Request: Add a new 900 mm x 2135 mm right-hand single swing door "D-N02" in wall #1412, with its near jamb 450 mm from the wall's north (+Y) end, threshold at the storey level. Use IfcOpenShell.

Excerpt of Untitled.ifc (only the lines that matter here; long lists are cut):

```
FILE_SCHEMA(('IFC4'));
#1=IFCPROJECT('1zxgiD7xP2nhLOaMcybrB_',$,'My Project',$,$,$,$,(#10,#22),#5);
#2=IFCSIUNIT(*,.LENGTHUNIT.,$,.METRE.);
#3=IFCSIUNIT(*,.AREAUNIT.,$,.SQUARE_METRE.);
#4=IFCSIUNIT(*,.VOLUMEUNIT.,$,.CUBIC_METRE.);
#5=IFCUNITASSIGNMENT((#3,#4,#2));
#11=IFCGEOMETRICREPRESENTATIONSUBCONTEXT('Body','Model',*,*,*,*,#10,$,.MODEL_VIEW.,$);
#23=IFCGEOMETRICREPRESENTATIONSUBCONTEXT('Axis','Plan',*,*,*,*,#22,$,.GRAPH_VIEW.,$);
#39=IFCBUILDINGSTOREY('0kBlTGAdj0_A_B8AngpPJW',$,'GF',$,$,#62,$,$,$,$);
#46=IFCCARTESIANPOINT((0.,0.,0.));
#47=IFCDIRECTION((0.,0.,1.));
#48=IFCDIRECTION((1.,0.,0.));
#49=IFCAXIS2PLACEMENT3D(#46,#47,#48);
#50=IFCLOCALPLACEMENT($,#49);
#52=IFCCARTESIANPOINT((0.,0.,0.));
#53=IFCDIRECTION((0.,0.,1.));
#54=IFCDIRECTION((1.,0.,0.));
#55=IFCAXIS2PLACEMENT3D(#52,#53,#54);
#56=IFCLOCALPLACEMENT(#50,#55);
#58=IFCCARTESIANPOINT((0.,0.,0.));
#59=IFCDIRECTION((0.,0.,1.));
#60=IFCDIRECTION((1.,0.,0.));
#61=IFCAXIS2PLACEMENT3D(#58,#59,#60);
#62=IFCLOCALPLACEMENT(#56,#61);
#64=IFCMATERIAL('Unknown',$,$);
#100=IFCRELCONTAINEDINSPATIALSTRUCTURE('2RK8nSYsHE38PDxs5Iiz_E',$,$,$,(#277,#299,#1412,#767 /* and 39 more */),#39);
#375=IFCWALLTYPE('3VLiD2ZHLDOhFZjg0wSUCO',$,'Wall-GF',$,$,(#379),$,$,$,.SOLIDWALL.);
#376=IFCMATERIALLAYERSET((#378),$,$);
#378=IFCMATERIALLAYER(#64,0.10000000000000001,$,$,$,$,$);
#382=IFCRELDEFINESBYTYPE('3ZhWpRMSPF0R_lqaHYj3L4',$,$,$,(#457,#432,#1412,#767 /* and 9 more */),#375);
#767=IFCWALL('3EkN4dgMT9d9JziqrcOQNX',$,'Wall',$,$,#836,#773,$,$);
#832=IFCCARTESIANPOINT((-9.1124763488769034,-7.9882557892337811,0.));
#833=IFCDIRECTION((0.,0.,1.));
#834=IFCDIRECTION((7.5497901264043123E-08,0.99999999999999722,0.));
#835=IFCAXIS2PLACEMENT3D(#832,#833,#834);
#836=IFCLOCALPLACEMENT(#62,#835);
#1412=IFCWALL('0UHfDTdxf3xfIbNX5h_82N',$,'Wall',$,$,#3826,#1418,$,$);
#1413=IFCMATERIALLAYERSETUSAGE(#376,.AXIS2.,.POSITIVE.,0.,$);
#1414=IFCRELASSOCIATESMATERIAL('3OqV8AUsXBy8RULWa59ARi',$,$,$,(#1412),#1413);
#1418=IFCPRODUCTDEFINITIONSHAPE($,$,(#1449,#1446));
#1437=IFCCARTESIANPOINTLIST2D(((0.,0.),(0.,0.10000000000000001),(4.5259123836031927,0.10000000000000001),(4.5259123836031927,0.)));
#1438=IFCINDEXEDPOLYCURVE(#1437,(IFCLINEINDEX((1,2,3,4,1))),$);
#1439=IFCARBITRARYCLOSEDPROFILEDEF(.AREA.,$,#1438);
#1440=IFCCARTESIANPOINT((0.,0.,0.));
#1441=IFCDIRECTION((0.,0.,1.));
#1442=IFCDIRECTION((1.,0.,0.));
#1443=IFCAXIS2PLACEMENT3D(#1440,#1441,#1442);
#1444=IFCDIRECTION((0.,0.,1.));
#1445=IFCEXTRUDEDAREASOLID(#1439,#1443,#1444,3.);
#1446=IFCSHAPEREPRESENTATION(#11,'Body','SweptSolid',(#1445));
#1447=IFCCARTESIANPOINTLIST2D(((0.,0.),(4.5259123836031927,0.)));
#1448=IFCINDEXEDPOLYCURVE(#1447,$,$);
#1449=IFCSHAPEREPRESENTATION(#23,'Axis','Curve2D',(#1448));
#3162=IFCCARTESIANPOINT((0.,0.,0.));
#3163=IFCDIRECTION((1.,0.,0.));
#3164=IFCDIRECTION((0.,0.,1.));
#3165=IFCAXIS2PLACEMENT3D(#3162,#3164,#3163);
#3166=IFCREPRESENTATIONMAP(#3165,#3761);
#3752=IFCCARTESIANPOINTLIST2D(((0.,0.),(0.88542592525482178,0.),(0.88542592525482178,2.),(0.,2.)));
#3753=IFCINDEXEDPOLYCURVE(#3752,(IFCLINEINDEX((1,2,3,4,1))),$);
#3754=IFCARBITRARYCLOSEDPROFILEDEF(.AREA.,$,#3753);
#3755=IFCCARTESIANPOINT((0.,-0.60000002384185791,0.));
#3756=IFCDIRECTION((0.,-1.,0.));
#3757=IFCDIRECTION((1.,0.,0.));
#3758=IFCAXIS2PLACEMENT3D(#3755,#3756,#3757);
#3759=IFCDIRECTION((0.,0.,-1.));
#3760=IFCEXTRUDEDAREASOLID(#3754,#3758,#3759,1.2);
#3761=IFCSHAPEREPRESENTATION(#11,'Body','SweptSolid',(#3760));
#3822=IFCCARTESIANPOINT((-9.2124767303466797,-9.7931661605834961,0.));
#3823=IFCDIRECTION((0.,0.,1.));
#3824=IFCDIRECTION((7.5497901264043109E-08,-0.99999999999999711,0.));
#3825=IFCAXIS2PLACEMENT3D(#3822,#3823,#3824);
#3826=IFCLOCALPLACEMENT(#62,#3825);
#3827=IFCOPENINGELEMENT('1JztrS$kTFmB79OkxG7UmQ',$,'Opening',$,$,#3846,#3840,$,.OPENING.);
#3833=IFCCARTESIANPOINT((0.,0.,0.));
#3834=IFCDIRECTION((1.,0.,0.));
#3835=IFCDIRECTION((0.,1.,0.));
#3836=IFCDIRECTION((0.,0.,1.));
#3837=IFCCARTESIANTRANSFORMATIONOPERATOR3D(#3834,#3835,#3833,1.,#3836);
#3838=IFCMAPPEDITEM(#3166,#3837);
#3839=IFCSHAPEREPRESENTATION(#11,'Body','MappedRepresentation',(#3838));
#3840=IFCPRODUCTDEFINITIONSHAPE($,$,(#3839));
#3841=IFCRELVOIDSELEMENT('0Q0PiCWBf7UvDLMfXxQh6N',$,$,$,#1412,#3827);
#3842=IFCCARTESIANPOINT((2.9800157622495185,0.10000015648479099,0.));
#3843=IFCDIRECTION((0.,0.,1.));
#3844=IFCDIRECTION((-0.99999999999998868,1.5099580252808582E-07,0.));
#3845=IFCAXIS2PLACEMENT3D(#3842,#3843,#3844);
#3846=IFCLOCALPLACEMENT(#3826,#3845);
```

```python
import numpy as np
import ifcopenshell
import ifcopenshell.api.feature
import ifcopenshell.api.geometry
import ifcopenshell.api.root
import ifcopenshell.api.spatial
import ifcopenshell.geom
import ifcopenshell.util.element
import ifcopenshell.util.placement
import ifcopenshell.util.representation
import ifcopenshell.util.shape
import ifcopenshell.util.unit

model = ifcopenshell.open("Untitled.ifc")
unit_scale = ifcopenshell.util.unit.calculate_unit_scale(model)
settings = ifcopenshell.geom.settings()


def volume(element):
    """Net volume in cubic metres, openings subtracted."""
    shape = ifcopenshell.geom.create_shape(settings, element)
    return ifcopenshell.util.shape.get_volume(shape.geometry)


wall = model.by_id(1412)
storey = ifcopenshell.util.element.get_container(wall, ifc_class="IfcBuildingStorey")
context = ifcopenshell.util.representation.get_context(model, "Model", "Body", "MODEL_VIEW")
before = volume(wall)

width, height, from_end, sill = 0.9, 2.135, 0.45, 0.0  # metres

# The wall runs along its own X axis, and the end named is its -X end.
wall_shape = ifcopenshell.geom.create_shape(settings, wall)
x, y, z = ifcopenshell.util.shape.get_vertices(wall_shape.geometry).T
start = x.min() + from_end
face, thickness = float(y.min()), float(y.max() - y.min())
wall_matrix = ifcopenshell.util.placement.get_local_placement(wall.ObjectPlacement)
level = ifcopenshell.util.placement.get_local_placement(storey.ObjectPlacement)[2, 3]


def in_wall(x, y):
    """Placement at x, y metres in the wall's axes, at sill height."""
    matrix = wall_matrix.copy()
    matrix[:, 3] = wall_matrix @ np.array([x / unit_scale, y / unit_scale, 0.0, 1.0])
    matrix[2, 3] = level + sill / unit_scale
    return matrix


# Opening: a box that overshoots both wall faces by 50 mm.
opening = ifcopenshell.api.root.create_entity(model, ifc_class="IfcOpeningElement", predefined_type="OPENING")
box = ifcopenshell.api.geometry.add_wall_representation(
    model, context=context, length=width, height=height, thickness=thickness + 0.1
)
ifcopenshell.api.geometry.assign_representation(model, product=opening, representation=box)
ifcopenshell.api.geometry.edit_object_placement(model, product=opening, matrix=in_wall(start, face - 0.05), is_si=False)
ifcopenshell.api.feature.add_feature(model, feature=opening, element=wall)

door = ifcopenshell.api.root.create_entity(model, ifc_class="IfcDoor", name="D-N02", predefined_type="DOOR")
door.OverallWidth, door.OverallHeight = width / unit_scale, height / unit_scale
door.OperationType = "SINGLE_SWING_RIGHT"
body = ifcopenshell.api.geometry.add_door_representation(
    model,
    context=context,
    overall_width=door.OverallWidth,
    overall_height=door.OverallHeight,
    operation_type="SINGLE_SWING_RIGHT",
    lining_properties={"LiningDepth": thickness / unit_scale, "ThresholdDepth": thickness / unit_scale},
)
ifcopenshell.api.geometry.assign_representation(model, product=door, representation=body)
ifcopenshell.api.spatial.assign_container(model, products=[door], relating_structure=storey)
ifcopenshell.api.feature.add_filling(model, opening=opening, element=door)

# The lining spans the wall, so the door starts at the wall face.
ifcopenshell.api.geometry.edit_object_placement(model, product=door, matrix=in_wall(start, face), is_si=False)

after = volume(wall)

print(f"wall volume {before:.3f} -> {after:.3f} m3")

model.write("Untitled_rev.ifc")
```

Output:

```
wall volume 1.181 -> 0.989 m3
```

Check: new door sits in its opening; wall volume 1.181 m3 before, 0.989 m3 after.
